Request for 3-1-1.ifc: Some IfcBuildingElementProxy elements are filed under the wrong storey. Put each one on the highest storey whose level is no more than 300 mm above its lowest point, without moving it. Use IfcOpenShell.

First a look at what the model holds.

```python
import ifcopenshell
import ifcopenshell.util.element
import ifcopenshell.util.placement

model = ifcopenshell.open("3-1-1.ifc")
print(model.schema)
for storey in model.by_type("IfcBuildingStorey"):
    level = ifcopenshell.util.placement.get_storey_elevation(storey)
    count = sum(e.is_a("IfcBuildingElementProxy") for e in ifcopenshell.util.element.get_contained(storey))
    print(storey.id(), storey.Name, round(level, 3), count, sep=" | ")
```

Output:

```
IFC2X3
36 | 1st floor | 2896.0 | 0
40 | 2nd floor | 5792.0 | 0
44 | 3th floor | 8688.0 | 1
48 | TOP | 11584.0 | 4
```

```python
import ifcopenshell
import ifcopenshell.api.spatial
import ifcopenshell.geom
import ifcopenshell.util.element
import ifcopenshell.util.placement
import ifcopenshell.util.shape
import ifcopenshell.util.unit

model = ifcopenshell.open("3-1-1.ifc")
unit_scale = ifcopenshell.util.unit.calculate_unit_scale(model)
settings = ifcopenshell.geom.settings()

levels = sorted(
    ((ifcopenshell.util.placement.get_storey_elevation(s) * unit_scale, s) for s in model.by_type("IfcBuildingStorey")),
    key=lambda pair: pair[0],
)

for e in model.by_type("IfcBuildingElementProxy"):
    current = e.ContainedInStructure[0].RelatingStructure if e.ContainedInStructure else None
    if current is None or not current.is_a("IfcBuildingStorey"):
        continue
    shape = ifcopenshell.geom.create_shape(settings, e)
    bottom = ifcopenshell.util.shape.get_shape_bottom_elevation(shape, shape.geometry)
    below = [s for level, s in levels if level <= bottom + 0.3]
    storey = below[-1] if below else levels[0][1]
    if storey != current:
        # assign_container keeps the world position.
        ifcopenshell.api.spatial.assign_container(model, products=[e], relating_structure=storey)
        print(e.id(), current.Name, "->", storey.Name)

model.write("3-1-1_updated.ifc")
```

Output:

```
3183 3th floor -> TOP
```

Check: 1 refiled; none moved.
